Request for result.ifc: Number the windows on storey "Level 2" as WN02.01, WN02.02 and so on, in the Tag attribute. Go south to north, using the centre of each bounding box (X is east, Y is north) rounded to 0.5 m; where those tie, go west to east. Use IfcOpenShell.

First a look at what the model holds.

```python
import ifcopenshell
import ifcopenshell.util.element
import ifcopenshell.util.placement

model = ifcopenshell.open("result.ifc")
print(model.schema)
storey = next(s for s in model.by_type("IfcBuildingStorey") if s.Name == "Level 2")
windows = [e for e in ifcopenshell.util.element.get_decomposition(storey) if e.is_a("IfcWindow")]
for e in sorted(windows, key=lambda e: e.id()):
    origin = ifcopenshell.util.placement.get_local_placement(e.ObjectPlacement)[:3, 3]
    print(e.id(), e.Tag, e.Name, origin.round(2) + 0.0, sep=" | ")
```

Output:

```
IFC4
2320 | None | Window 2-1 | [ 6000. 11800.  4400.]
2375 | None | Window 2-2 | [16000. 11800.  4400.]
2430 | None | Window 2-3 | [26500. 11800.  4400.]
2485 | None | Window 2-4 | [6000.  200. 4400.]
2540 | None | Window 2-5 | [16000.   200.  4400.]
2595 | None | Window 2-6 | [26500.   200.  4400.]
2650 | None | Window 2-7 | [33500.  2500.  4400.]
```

```python
import ifcopenshell
import ifcopenshell.geom
import ifcopenshell.util.element
import ifcopenshell.util.shape

model = ifcopenshell.open("result.ifc")
settings = ifcopenshell.geom.settings()
settings.set("use-world-coords", True)


def centre(element):
    shape = ifcopenshell.geom.create_shape(settings, element)
    return ifcopenshell.util.shape.get_bbox_centroid(shape.geometry)


storey = next(s for s in model.by_type("IfcBuildingStorey") if s.Name == "Level 2")
windows = [e for e in ifcopenshell.util.element.get_decomposition(storey) if e.is_a("IfcWindow")]

# Insertion points can sit at a corner or the storey origin, so sort by the geometry (in metres).
centres = {e: centre(e) for e in windows}
windows.sort(key=lambda e: (round(centres[e][1] / 0.5), centres[e][0]))

for i, e in enumerate(windows, start=1):
    number = f"WN02.{i:02d}"
    e.Tag = number
    print(e.id(), number)

model.write("result_v2.ifc")
```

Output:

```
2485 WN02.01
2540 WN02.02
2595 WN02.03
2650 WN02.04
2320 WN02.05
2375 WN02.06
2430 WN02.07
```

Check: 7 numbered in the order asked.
